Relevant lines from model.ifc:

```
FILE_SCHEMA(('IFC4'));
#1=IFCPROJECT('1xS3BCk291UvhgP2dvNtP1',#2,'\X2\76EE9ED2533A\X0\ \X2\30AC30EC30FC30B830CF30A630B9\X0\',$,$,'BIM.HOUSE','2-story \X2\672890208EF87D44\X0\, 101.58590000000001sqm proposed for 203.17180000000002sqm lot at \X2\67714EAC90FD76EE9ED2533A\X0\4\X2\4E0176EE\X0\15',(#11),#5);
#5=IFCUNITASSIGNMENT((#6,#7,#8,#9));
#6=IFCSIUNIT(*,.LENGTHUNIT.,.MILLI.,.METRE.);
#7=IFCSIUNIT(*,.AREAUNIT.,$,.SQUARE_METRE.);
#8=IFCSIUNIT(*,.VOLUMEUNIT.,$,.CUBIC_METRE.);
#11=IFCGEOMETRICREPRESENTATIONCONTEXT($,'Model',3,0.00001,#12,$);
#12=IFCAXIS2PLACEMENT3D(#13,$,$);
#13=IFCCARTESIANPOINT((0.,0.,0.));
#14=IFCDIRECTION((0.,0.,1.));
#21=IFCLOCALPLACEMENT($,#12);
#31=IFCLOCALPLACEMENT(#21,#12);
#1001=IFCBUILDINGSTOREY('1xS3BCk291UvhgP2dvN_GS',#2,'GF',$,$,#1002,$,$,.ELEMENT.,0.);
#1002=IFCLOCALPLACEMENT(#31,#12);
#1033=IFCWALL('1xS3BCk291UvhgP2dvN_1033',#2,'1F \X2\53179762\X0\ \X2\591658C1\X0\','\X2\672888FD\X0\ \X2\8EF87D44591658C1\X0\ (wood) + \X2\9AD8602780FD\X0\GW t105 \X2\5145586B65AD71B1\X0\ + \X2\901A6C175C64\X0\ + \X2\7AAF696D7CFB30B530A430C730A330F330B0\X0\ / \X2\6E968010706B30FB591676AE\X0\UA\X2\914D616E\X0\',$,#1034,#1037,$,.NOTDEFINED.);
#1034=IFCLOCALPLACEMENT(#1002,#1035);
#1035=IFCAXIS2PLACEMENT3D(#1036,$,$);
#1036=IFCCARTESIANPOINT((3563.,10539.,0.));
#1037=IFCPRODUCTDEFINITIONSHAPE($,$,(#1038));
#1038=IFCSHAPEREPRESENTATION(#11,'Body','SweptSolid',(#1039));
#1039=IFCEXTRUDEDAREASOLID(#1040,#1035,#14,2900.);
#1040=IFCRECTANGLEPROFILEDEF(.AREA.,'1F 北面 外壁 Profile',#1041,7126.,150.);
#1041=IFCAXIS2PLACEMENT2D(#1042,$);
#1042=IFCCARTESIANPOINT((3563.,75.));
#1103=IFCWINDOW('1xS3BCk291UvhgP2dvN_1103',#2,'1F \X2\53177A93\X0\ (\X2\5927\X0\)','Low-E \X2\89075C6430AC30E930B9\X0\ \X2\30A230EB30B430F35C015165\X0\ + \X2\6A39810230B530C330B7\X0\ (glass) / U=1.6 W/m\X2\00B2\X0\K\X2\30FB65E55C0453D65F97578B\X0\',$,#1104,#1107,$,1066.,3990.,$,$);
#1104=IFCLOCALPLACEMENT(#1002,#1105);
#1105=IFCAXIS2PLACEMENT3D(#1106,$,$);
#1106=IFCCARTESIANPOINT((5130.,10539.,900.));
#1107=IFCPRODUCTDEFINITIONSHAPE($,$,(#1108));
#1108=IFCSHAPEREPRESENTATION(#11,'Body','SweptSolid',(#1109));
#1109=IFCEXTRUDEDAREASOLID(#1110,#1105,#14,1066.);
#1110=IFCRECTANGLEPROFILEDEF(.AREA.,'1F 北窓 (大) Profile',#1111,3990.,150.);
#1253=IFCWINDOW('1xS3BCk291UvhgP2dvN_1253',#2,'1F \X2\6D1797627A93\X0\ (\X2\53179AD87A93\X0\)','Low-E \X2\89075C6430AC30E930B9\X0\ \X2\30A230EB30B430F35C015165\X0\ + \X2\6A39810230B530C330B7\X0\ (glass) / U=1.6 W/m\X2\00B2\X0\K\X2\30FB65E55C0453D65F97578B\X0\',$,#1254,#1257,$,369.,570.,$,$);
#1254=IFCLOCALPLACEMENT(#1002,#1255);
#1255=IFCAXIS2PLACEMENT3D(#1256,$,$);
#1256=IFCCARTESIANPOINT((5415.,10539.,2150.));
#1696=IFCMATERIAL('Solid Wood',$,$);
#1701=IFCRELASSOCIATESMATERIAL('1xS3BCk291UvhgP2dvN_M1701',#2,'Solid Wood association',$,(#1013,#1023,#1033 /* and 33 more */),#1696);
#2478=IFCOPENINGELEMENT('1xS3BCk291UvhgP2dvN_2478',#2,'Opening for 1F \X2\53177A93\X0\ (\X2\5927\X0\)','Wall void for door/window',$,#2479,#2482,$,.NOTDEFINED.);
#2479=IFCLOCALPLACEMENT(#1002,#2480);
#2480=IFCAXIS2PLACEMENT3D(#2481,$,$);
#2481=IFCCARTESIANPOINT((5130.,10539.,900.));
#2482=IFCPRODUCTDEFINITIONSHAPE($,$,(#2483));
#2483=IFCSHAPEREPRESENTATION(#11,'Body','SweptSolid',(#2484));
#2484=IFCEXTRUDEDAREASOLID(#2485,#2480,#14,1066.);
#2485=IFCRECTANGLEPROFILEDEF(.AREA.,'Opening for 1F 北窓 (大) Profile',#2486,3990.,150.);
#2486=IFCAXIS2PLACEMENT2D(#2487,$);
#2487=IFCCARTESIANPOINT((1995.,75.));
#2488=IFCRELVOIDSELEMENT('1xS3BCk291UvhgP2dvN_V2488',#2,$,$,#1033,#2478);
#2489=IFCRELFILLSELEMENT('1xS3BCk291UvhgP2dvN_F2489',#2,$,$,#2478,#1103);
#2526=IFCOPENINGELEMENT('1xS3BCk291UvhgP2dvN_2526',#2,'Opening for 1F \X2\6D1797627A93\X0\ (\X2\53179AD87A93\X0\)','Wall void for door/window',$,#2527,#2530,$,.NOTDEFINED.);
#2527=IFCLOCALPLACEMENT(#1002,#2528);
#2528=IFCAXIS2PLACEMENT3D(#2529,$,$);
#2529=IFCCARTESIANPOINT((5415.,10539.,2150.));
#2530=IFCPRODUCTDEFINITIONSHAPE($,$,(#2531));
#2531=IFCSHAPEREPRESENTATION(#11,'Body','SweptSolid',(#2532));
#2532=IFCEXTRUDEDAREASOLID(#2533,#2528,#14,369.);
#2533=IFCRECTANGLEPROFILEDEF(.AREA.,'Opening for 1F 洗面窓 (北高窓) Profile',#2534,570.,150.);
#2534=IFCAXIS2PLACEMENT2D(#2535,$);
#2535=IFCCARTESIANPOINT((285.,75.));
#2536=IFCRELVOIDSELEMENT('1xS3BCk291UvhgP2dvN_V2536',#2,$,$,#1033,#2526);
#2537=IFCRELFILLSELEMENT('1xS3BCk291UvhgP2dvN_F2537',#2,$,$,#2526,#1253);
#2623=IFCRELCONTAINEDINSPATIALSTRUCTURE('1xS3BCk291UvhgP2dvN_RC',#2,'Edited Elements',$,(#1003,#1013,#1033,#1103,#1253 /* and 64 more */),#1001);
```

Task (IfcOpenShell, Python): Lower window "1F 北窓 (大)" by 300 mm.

```python
import numpy as np
import ifcopenshell
import ifcopenshell.api.geometry
import ifcopenshell.util.placement
import ifcopenshell.util.unit

model = ifcopenshell.open("model.ifc")
unit_scale = ifcopenshell.util.unit.calculate_unit_scale(model)

window = model.by_id(1103)
opening = window.FillsVoids[0].RelatingOpeningElement
dz = -0.3 / unit_scale

shift = np.array([0.0, 0.0, dz])
# The window is not placed relative to its opening, so move both.
for product in (opening, window):
    matrix = ifcopenshell.util.placement.get_local_placement(product.ObjectPlacement)
    matrix[:3, 3] += shift
    ifcopenshell.api.geometry.edit_object_placement(model, product=product, matrix=matrix, is_si=False)

print(f"moved by {dz * unit_scale:+.3f} m")

model.write("model_rev.ifc")
```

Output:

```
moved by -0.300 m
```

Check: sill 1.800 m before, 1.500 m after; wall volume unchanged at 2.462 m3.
